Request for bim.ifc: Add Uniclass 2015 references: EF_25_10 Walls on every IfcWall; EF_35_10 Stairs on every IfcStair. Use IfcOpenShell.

First a look at what the model holds.

```python
import ifcopenshell

model = ifcopenshell.open("bim.ifc")
print(model.schema)
print("classifications:", [c.Name for c in model.by_type("IfcClassification")])
for ifc_class in ("IfcDoor", "IfcRoof", "IfcStair", "IfcWall", "IfcWindow"):
    print(ifc_class, len(model.by_type(ifc_class)))
```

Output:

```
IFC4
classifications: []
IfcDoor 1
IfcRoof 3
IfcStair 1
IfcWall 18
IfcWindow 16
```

```python
import ifcopenshell
import ifcopenshell.api.classification

model = ifcopenshell.open("bim.ifc")

system = ifcopenshell.api.classification.add_classification(model, classification="Uniclass 2015")

codes = {
    "IfcWall": ("EF_25_10", "Walls"),
    "IfcStair": ("EF_35_10", "Stairs"),
}
for ifc_class, (code, name) in codes.items():
    products = model.by_type(ifc_class)
    ifcopenshell.api.classification.add_reference(
        model, products=products, classification=system, identification=code, name=name
    )
    print(code, len(products))

model.write("bim_updated.ifc")
```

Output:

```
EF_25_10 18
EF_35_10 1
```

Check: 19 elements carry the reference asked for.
